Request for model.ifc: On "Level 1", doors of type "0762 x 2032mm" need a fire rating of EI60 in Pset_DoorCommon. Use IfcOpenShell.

First a look at what the model holds.

```python
import ifcopenshell
import ifcopenshell.util.element

model = ifcopenshell.open("model.ifc")
print(model.schema)
storey = next(s for s in model.by_type("IfcBuildingStorey") if s.Name == "Level 1")
doors = [e for e in ifcopenshell.util.element.get_decomposition(storey) if e.is_a("IfcDoor")]
seen = {}
for e in doors:
    element_type = ifcopenshell.util.element.get_type(e)
    key = (element_type.Name if element_type != e and element_type else None, ifcopenshell.util.element.get_pset(e, "Pset_DoorCommon", "FireRating"))
    seen[key] = seen.get(key, 0) + 1
for (name, value), count in sorted(seen.items(), key=str):
    print(count, "x", name, "|", value)
```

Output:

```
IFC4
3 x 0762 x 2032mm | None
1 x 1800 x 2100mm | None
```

```python
import ifcopenshell
import ifcopenshell.api.pset
import ifcopenshell.util.element

model = ifcopenshell.open("model.ifc")

storey = next(s for s in model.by_type("IfcBuildingStorey") if s.Name == "Level 1")
doors = [e for e in ifcopenshell.util.element.get_decomposition(storey) if e.is_a("IfcDoor")]

count = 0
for e in doors:
    element_type = ifcopenshell.util.element.get_type(e)
    if element_type in (None, e) or element_type.Name != "0762 x 2032mm":
        continue
    # add_pset returns the element's existing set when there is one.
    pset = ifcopenshell.api.pset.add_pset(model, product=e, name="Pset_DoorCommon")
    ifcopenshell.api.pset.edit_pset(model, pset=pset, properties={"FireRating": "EI60"})
    count += 1

print(count, "doors updated")

model.write("model_rev.ifc")
```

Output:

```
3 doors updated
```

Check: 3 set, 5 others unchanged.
